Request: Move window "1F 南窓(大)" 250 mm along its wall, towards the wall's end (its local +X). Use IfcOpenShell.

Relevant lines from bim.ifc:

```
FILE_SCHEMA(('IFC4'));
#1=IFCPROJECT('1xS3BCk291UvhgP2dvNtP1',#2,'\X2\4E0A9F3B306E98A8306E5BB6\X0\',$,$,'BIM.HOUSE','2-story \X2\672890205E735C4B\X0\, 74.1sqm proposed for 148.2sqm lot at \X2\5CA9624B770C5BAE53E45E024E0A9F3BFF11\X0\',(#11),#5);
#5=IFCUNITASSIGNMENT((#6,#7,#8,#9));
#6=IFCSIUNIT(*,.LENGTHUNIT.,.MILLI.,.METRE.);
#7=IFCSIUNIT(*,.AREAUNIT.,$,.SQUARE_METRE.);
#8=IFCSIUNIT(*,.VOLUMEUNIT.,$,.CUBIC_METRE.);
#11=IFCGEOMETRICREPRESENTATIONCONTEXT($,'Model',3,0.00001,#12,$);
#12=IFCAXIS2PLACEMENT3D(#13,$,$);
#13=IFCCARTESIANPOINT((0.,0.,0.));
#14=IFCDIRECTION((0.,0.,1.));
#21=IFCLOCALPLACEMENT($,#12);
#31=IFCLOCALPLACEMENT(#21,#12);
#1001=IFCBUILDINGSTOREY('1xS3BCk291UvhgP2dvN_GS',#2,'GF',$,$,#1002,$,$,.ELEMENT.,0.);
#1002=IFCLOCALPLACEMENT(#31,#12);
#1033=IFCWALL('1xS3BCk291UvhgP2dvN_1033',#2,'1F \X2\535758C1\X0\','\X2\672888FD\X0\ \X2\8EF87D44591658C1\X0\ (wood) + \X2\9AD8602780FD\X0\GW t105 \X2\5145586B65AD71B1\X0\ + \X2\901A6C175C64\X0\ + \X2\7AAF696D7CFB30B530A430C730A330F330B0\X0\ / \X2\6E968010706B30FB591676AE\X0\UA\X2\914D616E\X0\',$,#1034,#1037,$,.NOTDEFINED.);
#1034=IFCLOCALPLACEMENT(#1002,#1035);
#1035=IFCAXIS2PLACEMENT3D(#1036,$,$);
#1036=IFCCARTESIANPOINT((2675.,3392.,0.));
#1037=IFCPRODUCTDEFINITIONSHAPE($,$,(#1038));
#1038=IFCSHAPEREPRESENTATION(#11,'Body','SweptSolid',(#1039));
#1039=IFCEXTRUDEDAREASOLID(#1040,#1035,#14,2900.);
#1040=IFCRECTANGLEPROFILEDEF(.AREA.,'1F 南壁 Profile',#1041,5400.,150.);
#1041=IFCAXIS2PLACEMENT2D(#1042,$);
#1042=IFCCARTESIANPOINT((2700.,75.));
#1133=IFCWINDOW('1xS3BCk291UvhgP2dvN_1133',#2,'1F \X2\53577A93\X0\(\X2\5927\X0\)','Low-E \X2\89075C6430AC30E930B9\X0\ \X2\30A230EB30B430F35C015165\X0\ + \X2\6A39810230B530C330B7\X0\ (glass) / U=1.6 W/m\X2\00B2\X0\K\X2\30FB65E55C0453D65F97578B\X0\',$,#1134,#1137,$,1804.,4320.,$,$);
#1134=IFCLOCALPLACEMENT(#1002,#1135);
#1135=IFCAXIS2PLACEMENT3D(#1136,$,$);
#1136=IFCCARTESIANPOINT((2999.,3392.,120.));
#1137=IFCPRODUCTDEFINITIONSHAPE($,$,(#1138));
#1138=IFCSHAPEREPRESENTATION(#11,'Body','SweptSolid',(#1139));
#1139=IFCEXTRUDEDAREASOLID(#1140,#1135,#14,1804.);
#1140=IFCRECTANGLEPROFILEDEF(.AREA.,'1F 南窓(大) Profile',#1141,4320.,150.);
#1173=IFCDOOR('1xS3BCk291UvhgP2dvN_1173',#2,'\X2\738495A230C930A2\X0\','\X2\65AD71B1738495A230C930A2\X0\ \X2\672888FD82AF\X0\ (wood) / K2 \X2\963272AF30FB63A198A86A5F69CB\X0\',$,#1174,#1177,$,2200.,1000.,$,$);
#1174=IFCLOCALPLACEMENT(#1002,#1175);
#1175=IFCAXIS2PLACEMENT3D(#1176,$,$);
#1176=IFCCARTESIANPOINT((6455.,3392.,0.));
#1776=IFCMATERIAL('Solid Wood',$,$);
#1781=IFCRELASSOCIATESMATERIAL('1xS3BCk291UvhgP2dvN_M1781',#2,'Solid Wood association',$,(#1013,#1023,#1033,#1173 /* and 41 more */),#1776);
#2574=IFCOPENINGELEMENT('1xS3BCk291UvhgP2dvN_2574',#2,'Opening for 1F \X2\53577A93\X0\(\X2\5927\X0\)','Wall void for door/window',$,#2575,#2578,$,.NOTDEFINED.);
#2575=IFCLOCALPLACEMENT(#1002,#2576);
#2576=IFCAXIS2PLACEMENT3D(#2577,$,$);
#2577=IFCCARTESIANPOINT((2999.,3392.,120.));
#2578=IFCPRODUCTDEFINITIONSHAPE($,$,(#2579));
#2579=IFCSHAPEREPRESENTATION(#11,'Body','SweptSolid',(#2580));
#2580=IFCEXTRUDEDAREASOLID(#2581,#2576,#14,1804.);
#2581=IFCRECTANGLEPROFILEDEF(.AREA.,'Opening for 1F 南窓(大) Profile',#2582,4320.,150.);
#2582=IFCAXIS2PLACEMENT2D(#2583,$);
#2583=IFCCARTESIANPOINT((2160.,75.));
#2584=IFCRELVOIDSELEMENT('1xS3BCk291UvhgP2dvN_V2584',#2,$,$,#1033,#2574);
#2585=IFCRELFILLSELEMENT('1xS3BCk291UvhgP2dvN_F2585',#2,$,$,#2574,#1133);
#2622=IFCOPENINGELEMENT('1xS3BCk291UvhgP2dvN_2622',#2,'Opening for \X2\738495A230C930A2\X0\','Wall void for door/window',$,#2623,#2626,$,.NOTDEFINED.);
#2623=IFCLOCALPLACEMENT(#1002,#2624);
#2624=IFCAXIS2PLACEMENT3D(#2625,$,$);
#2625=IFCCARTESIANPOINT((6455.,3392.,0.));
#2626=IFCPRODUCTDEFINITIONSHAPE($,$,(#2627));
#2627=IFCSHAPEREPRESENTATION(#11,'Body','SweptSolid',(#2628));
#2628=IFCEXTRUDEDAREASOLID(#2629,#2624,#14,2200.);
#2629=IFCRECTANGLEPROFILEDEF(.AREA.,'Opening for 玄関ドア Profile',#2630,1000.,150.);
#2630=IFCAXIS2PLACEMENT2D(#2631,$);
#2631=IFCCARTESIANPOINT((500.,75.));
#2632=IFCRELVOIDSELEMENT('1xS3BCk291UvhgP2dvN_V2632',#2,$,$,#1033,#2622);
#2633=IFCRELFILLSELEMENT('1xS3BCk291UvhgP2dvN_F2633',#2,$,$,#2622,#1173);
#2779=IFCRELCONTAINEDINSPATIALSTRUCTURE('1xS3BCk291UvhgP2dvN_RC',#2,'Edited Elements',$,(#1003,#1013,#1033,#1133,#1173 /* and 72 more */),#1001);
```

```python
import ifcopenshell
import ifcopenshell.api.geometry
import ifcopenshell.util.placement
import ifcopenshell.util.unit

model = ifcopenshell.open("bim.ifc")
unit_scale = ifcopenshell.util.unit.calculate_unit_scale(model)

window = model.by_id(1133)
opening = window.FillsVoids[0].RelatingOpeningElement
wall = opening.VoidsElements[0].RelatingBuildingElement

wall_matrix = ifcopenshell.util.placement.get_local_placement(wall.ObjectPlacement)
shift = wall_matrix[:3, 0] * 0.25 / unit_scale
before = ifcopenshell.util.placement.get_local_placement(window.ObjectPlacement)[:3, 3].copy()

# The window is not placed relative to its opening, so move both.
for product in (opening, window):
    matrix = ifcopenshell.util.placement.get_local_placement(product.ObjectPlacement)
    matrix[:3, 3] += shift
    ifcopenshell.api.geometry.edit_object_placement(model, product=product, matrix=matrix, is_si=False)

after = ifcopenshell.util.placement.get_local_placement(window.ObjectPlacement)[:3, 3]
print("window moved by", (after - before).round(3) + 0.0)

model.write("bim_updated.ifc")
```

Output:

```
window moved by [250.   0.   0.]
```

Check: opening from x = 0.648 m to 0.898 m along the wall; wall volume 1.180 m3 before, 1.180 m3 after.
